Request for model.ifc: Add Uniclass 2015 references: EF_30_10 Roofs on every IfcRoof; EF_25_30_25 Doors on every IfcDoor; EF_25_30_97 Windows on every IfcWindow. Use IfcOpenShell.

First a look at what the model holds.

```python
import ifcopenshell

model = ifcopenshell.open("model.ifc")
print(model.schema)
print("classifications:", [c.Name for c in model.by_type("IfcClassification")])
for ifc_class in ("IfcDoor", "IfcRoof", "IfcStair", "IfcWall", "IfcWindow"):
    print(ifc_class, len(model.by_type(ifc_class)))
```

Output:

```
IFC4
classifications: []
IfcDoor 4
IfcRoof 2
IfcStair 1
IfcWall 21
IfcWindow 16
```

```python
import ifcopenshell
import ifcopenshell.api.classification

model = ifcopenshell.open("model.ifc")

system = ifcopenshell.api.classification.add_classification(model, classification="Uniclass 2015")

codes = {
    "IfcRoof": ("EF_30_10", "Roofs"),
    "IfcDoor": ("EF_25_30_25", "Doors"),
    "IfcWindow": ("EF_25_30_97", "Windows"),
}
for ifc_class, (code, name) in codes.items():
    products = model.by_type(ifc_class)
    ifcopenshell.api.classification.add_reference(
        model, products=products, classification=system, identification=code, name=name
    )
    print(code, len(products))

model.write("model_rev.ifc")
```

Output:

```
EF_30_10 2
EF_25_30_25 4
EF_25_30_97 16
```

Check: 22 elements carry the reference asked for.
